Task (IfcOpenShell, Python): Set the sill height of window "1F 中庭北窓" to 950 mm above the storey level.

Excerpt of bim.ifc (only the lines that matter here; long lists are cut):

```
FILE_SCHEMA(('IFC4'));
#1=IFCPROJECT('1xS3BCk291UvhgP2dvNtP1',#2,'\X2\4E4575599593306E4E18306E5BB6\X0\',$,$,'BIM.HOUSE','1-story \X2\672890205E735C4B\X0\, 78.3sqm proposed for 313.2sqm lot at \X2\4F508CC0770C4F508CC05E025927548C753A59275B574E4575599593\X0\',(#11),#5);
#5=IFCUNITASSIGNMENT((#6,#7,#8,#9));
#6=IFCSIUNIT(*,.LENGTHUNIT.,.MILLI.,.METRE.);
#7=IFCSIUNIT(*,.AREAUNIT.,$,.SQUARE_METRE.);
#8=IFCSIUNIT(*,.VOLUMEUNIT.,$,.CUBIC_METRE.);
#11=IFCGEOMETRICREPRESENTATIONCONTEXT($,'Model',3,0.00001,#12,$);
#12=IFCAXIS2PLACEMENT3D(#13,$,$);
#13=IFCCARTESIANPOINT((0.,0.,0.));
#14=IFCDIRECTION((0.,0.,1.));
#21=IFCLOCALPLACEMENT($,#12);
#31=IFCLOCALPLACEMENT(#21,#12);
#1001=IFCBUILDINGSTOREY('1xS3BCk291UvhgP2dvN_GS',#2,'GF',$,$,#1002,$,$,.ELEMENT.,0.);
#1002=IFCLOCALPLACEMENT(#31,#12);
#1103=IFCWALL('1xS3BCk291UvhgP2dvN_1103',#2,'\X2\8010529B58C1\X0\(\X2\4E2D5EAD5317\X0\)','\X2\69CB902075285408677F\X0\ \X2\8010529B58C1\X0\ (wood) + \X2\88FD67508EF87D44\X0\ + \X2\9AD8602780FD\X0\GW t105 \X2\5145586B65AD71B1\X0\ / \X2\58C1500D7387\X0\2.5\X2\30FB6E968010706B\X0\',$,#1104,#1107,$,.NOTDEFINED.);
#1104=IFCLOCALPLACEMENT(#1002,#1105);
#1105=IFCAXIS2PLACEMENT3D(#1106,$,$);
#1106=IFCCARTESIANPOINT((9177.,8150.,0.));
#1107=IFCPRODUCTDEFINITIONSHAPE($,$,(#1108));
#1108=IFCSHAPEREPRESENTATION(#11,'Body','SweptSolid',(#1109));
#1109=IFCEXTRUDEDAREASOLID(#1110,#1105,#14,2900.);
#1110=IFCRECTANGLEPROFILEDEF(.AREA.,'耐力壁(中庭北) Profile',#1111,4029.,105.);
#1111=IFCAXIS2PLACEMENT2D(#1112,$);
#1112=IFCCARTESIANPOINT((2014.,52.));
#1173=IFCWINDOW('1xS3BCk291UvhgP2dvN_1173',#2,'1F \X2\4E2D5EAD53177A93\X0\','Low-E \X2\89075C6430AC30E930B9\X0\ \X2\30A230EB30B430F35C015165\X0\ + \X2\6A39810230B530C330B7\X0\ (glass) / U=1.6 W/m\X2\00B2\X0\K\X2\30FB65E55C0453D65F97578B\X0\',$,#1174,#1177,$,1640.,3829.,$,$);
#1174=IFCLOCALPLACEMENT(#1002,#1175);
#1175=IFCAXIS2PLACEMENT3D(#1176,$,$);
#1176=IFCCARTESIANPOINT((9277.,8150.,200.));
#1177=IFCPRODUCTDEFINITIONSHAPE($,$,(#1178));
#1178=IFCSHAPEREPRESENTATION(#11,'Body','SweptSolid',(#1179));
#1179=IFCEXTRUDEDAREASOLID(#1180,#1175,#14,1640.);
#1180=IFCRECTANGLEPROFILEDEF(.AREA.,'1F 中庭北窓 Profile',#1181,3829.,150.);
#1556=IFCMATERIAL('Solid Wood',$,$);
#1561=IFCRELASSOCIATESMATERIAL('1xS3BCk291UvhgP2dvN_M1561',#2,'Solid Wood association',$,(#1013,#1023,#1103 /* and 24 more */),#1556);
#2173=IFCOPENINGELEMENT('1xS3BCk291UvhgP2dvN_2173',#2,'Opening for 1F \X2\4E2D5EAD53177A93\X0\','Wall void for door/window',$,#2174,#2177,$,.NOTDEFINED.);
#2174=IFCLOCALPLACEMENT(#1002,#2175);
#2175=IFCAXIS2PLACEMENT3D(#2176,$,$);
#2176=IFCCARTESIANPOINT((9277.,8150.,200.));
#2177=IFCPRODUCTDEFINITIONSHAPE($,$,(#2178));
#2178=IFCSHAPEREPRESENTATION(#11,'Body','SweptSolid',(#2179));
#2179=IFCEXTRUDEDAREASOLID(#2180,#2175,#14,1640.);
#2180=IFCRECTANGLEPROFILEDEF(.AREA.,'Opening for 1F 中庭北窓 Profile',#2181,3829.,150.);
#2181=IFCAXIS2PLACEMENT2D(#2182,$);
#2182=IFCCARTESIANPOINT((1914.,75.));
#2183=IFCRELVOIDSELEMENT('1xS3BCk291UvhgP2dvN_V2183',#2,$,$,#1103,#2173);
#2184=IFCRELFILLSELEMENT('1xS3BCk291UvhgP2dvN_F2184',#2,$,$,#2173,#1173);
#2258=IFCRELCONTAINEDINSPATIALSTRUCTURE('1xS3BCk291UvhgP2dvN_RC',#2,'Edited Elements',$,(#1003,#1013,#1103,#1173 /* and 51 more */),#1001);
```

```python
import numpy as np
import ifcopenshell
import ifcopenshell.api.geometry
import ifcopenshell.geom
import ifcopenshell.util.element
import ifcopenshell.util.placement
import ifcopenshell.util.shape
import ifcopenshell.util.unit

model = ifcopenshell.open("bim.ifc")
unit_scale = ifcopenshell.util.unit.calculate_unit_scale(model)

window = model.by_guid("1xS3BCk291UvhgP2dvN_1173")
opening = window.FillsVoids[0].RelatingOpeningElement
storey = ifcopenshell.util.element.get_container(window, ifc_class="IfcBuildingStorey")
level = ifcopenshell.util.placement.get_local_placement(storey.ObjectPlacement)[2, 3]

# The opening's origin need not be at the sill, so measure its lowest point.
shape = ifcopenshell.geom.create_shape(ifcopenshell.geom.settings(), opening)
bottom = ifcopenshell.util.shape.get_shape_bottom_elevation(shape, shape.geometry) / unit_scale
dz = level + 0.95 / unit_scale - bottom

shift = np.array([0.0, 0.0, dz])
# The window is not placed relative to its opening, so move both.
for product in (opening, window):
    matrix = ifcopenshell.util.placement.get_local_placement(product.ObjectPlacement)
    matrix[:3, 3] += shift
    ifcopenshell.api.geometry.edit_object_placement(model, product=product, matrix=matrix, is_si=False)

print(f"moved by {dz * unit_scale:+.3f} m")

model.write("bim_v2.ifc")
```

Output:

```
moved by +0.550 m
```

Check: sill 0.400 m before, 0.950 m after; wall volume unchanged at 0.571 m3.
